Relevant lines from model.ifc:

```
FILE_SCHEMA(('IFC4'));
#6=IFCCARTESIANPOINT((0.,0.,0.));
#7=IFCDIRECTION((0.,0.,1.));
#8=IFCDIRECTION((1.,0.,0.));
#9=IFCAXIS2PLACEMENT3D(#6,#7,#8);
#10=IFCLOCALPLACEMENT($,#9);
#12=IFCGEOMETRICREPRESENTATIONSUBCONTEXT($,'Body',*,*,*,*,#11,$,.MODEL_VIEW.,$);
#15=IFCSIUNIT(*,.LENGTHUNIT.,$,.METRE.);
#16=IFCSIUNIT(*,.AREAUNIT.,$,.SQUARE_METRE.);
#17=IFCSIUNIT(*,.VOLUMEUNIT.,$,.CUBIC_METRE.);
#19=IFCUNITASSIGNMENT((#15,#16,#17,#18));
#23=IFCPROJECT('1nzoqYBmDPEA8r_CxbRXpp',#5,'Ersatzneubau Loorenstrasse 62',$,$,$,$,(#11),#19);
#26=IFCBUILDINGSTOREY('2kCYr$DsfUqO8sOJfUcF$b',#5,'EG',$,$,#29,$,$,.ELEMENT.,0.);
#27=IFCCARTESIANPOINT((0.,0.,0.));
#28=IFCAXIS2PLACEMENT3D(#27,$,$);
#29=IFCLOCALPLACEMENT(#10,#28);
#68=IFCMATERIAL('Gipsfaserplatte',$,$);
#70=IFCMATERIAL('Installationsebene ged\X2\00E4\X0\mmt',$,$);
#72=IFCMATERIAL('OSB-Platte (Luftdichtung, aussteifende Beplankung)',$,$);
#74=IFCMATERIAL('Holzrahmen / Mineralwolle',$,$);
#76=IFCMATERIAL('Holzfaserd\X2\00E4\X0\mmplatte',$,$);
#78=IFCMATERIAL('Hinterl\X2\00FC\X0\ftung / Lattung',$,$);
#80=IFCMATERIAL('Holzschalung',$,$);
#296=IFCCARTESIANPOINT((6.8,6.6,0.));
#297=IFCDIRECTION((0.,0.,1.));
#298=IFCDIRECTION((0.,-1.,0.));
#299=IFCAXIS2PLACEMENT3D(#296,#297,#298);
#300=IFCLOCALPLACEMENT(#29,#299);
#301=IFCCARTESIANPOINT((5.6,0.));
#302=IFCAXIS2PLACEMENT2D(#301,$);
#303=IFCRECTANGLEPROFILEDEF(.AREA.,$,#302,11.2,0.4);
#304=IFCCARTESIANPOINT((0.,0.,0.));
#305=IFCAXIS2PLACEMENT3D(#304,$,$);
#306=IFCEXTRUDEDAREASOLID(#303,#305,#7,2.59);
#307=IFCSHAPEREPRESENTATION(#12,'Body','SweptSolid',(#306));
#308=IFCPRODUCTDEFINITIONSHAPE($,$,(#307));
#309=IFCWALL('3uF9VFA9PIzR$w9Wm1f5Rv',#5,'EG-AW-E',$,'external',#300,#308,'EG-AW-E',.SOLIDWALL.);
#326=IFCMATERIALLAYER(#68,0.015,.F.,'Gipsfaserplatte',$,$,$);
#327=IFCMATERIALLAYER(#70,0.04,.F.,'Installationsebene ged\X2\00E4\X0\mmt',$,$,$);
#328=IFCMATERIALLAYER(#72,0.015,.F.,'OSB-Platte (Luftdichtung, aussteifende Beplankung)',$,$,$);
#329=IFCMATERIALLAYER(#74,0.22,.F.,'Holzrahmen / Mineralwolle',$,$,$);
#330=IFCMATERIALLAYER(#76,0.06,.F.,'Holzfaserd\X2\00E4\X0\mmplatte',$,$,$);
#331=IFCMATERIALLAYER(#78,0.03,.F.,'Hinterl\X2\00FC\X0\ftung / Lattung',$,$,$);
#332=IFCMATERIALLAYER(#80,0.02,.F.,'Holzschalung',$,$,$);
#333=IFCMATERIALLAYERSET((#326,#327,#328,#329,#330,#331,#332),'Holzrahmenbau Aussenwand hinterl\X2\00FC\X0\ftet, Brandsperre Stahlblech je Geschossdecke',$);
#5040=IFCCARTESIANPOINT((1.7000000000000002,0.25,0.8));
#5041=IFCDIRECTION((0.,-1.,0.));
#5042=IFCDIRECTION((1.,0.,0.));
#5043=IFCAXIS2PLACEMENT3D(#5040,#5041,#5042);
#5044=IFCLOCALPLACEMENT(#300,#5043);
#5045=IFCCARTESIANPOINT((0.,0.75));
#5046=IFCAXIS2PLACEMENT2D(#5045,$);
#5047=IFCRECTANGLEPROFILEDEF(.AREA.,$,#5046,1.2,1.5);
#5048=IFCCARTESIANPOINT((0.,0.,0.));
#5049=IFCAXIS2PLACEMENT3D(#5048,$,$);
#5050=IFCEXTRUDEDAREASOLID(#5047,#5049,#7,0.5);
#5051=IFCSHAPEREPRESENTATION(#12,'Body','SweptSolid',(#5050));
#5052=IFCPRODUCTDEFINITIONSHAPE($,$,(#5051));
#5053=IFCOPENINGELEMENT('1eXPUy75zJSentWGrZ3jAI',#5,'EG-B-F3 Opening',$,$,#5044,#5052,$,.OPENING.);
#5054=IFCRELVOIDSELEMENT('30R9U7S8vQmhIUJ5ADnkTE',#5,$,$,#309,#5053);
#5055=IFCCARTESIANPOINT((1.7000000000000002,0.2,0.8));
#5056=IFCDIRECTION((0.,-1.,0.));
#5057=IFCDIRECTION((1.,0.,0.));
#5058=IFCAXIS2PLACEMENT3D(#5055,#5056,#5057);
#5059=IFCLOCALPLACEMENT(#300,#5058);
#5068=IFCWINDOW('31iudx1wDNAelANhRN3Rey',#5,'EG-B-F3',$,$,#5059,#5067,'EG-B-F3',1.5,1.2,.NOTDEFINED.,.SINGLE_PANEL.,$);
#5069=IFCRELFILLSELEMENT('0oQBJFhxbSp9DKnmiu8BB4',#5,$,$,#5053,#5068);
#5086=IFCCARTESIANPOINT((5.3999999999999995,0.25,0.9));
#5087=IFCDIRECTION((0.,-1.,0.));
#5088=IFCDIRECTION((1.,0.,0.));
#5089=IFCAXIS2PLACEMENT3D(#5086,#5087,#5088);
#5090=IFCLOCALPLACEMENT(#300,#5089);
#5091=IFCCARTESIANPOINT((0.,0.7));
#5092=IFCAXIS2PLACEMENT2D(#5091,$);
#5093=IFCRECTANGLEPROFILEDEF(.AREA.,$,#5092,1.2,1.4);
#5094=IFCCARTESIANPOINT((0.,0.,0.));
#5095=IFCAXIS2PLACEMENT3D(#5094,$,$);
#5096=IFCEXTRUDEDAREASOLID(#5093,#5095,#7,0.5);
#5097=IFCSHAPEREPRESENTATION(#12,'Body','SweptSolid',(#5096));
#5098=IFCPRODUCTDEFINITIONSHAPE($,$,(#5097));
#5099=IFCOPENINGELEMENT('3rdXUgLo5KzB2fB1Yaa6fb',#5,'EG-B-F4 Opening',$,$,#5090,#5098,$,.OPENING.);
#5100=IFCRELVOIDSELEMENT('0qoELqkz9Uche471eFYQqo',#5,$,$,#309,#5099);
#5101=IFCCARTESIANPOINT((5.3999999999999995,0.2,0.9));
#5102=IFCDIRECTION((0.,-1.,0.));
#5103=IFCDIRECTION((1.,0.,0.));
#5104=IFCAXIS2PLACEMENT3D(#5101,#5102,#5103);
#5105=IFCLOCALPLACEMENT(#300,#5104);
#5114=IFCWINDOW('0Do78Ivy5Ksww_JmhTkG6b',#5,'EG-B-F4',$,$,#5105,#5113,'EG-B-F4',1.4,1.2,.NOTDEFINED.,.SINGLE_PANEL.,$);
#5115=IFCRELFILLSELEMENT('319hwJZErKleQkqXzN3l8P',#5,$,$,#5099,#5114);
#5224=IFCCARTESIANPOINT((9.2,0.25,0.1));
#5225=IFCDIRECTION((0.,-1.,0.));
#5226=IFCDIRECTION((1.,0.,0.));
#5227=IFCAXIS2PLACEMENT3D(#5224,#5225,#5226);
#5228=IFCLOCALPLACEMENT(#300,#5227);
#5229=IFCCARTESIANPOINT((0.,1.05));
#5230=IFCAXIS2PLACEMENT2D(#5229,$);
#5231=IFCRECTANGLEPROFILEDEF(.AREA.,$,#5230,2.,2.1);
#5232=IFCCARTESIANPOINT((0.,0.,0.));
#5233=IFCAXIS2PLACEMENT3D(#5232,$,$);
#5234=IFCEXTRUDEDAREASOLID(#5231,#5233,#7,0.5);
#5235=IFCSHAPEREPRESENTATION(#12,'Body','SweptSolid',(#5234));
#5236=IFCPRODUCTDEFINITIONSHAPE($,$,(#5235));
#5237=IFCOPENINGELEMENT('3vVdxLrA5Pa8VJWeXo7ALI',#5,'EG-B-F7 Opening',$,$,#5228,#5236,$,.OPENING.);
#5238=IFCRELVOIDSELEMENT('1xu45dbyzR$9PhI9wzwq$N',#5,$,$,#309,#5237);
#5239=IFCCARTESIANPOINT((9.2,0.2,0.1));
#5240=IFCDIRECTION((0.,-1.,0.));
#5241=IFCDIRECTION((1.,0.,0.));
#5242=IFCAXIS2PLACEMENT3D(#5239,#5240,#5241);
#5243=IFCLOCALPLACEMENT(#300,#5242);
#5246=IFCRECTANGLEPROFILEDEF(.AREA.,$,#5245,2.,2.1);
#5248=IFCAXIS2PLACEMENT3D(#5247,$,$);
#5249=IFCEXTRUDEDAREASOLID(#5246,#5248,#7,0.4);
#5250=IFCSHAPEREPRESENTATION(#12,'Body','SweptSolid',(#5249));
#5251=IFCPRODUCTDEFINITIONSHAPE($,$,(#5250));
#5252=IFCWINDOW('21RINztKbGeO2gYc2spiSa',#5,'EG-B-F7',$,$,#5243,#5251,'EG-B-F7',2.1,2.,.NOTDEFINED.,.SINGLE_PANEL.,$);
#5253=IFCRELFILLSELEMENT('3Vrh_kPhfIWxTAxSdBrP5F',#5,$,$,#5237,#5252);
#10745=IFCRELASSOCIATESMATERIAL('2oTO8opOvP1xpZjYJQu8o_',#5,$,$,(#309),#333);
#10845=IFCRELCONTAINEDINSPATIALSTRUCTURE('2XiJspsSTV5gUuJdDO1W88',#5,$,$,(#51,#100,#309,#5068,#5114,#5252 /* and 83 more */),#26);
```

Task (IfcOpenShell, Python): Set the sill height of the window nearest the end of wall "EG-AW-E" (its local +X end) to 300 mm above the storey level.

```python
import numpy as np
import ifcopenshell
import ifcopenshell.api.geometry
import ifcopenshell.geom
import ifcopenshell.util.element
import ifcopenshell.util.placement
import ifcopenshell.util.shape
import ifcopenshell.util.unit

model = ifcopenshell.open("model.ifc")
unit_scale = ifcopenshell.util.unit.calculate_unit_scale(model)

window = model.by_guid("21RINztKbGeO2gYc2spiSa")
opening = window.FillsVoids[0].RelatingOpeningElement
storey = ifcopenshell.util.element.get_container(window, ifc_class="IfcBuildingStorey")
level = ifcopenshell.util.placement.get_local_placement(storey.ObjectPlacement)[2, 3]

# The opening's origin need not be at the sill, so measure its lowest point.
shape = ifcopenshell.geom.create_shape(ifcopenshell.geom.settings(), opening)
bottom = ifcopenshell.util.shape.get_shape_bottom_elevation(shape, shape.geometry) / unit_scale
dz = level + 0.3 / unit_scale - bottom

shift = np.array([0.0, 0.0, dz])
# The window is not placed relative to its opening, so move both.
for product in (opening, window):
    matrix = ifcopenshell.util.placement.get_local_placement(product.ObjectPlacement)
    matrix[:3, 3] += shift
    ifcopenshell.api.geometry.edit_object_placement(model, product=product, matrix=matrix, is_si=False)

print(f"moved by {dz * unit_scale:+.3f} m")

model.write("model_edited.ifc")
```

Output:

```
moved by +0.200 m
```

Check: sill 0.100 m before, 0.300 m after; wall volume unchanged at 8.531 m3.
